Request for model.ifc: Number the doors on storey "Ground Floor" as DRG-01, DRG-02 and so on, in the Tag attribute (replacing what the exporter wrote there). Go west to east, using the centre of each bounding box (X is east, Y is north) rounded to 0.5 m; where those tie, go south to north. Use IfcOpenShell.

First a look at what the model holds.

```python
import ifcopenshell
import ifcopenshell.util.element
import ifcopenshell.util.placement

model = ifcopenshell.open("model.ifc")
print(model.schema)
storey = next(s for s in model.by_type("IfcBuildingStorey") if s.Name == "Ground Floor")
doors = [e for e in ifcopenshell.util.element.get_decomposition(storey) if e.is_a("IfcDoor")]
for e in sorted(doors, key=lambda e: e.id()):
    origin = ifcopenshell.util.placement.get_local_placement(e.ObjectPlacement)[:3, 3]
    print(e.id(), e.Tag, e.Name, origin.round(2) + 0.0, sep=" | ")
```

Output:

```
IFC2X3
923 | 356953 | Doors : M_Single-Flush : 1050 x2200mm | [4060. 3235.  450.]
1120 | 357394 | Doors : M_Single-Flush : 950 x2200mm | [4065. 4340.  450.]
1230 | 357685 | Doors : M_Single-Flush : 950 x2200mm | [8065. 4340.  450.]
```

```python
import ifcopenshell
import ifcopenshell.geom
import ifcopenshell.util.element
import ifcopenshell.util.shape

model = ifcopenshell.open("model.ifc")
settings = ifcopenshell.geom.settings()
settings.set("use-world-coords", True)


def centre(element):
    shape = ifcopenshell.geom.create_shape(settings, element)
    return ifcopenshell.util.shape.get_bbox_centroid(shape.geometry)


storey = next(s for s in model.by_type("IfcBuildingStorey") if s.Name == "Ground Floor")
doors = [e for e in ifcopenshell.util.element.get_decomposition(storey) if e.is_a("IfcDoor")]

# Insertion points can sit at a corner or the storey origin, so sort by the geometry (in metres).
centres = {e: centre(e) for e in doors}
doors.sort(key=lambda e: (round(centres[e][0] / 0.5), centres[e][1]))

for i, e in enumerate(doors, start=1):
    number = f"DRG-{i:02d}"
    e.Tag = number
    print(e.id(), number)

model.write("model_updated.ifc")
```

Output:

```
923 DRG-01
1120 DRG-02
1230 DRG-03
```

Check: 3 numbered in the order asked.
